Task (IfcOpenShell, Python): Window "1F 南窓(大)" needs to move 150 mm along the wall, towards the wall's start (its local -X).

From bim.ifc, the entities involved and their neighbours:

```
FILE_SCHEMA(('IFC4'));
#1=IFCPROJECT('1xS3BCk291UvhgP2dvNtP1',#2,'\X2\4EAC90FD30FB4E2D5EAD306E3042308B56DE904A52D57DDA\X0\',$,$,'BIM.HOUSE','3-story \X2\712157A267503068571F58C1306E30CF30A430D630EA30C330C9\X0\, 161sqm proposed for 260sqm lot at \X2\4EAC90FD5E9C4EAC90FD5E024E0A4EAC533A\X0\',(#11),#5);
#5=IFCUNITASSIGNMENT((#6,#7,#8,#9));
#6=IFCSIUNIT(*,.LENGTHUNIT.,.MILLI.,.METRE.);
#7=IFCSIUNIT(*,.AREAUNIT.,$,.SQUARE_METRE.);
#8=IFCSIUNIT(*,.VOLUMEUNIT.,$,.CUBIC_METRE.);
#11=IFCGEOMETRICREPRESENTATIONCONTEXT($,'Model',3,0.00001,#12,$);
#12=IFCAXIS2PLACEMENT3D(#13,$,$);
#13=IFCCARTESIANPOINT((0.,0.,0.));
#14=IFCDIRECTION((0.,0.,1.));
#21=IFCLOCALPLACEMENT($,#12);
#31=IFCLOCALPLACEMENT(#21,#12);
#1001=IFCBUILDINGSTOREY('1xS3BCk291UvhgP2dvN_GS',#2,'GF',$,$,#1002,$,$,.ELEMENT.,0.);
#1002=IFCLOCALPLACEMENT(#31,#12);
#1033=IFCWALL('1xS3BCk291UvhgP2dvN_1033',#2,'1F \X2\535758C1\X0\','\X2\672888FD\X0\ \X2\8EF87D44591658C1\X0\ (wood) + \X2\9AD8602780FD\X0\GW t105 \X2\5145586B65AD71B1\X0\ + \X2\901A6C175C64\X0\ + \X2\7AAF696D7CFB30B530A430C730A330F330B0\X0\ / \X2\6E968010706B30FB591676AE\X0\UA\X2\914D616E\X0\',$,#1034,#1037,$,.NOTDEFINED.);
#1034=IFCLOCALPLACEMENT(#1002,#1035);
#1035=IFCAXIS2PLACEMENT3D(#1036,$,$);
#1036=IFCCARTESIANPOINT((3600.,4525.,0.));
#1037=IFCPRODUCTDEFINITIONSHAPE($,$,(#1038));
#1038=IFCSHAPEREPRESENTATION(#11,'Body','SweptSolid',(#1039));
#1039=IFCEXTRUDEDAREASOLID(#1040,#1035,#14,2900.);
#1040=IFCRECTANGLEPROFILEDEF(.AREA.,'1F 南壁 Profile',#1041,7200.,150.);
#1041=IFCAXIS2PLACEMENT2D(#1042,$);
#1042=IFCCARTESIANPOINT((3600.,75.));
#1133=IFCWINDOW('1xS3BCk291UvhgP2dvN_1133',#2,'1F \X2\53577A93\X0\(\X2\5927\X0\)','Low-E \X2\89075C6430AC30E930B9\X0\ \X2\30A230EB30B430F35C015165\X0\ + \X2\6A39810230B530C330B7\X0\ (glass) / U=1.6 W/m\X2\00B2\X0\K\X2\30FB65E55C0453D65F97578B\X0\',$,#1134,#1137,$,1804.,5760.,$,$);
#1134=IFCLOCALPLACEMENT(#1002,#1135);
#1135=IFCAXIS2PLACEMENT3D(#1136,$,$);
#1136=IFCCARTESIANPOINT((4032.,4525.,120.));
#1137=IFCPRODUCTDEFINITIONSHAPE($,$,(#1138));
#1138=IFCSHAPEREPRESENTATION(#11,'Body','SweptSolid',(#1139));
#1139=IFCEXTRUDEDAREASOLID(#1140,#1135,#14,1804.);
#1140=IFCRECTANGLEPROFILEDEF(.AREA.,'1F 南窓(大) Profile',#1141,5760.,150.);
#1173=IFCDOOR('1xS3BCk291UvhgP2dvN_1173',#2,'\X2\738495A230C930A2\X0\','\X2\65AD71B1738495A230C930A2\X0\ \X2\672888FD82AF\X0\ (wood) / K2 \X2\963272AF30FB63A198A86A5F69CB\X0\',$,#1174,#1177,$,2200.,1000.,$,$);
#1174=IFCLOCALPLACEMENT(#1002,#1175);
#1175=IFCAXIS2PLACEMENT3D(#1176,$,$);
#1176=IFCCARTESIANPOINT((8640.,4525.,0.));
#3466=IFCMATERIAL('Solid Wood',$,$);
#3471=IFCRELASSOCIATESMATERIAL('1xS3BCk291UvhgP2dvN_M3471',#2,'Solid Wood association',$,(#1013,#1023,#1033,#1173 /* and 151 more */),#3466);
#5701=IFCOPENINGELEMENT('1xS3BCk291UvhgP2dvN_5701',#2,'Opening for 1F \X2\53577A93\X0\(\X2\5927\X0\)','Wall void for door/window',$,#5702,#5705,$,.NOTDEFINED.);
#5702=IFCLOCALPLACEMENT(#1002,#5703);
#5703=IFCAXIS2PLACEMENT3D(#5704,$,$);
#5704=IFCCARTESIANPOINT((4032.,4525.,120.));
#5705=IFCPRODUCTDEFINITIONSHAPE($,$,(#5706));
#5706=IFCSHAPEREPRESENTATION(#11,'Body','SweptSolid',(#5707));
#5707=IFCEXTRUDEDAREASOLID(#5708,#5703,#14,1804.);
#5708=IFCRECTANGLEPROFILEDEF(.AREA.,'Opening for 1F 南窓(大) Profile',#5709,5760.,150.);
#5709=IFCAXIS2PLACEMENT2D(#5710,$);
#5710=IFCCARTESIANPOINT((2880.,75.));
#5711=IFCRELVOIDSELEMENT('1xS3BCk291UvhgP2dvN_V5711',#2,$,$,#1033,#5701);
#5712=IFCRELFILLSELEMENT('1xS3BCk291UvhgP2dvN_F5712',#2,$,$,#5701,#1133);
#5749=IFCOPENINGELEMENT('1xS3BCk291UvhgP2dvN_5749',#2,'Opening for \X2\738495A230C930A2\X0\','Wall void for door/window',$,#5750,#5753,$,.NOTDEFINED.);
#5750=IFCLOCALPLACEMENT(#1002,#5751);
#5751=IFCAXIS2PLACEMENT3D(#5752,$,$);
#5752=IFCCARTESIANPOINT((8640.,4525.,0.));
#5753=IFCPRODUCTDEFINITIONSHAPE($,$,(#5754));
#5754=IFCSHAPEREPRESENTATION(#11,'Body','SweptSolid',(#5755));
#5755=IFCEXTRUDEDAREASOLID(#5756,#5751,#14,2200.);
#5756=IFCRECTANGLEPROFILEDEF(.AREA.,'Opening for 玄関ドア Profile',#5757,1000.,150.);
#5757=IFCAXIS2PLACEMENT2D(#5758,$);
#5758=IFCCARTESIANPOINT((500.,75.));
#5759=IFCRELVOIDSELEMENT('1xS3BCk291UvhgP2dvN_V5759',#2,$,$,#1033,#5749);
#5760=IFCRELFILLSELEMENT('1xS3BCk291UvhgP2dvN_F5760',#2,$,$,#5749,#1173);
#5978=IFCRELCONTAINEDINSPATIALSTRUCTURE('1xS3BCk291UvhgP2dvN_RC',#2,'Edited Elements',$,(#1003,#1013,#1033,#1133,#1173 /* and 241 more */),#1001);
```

```python
import ifcopenshell
import ifcopenshell.api.geometry
import ifcopenshell.util.placement

model = ifcopenshell.open("bim.ifc")

window = model.by_guid("1xS3BCk291UvhgP2dvN_1133")
opening = window.FillsVoids[0].RelatingOpeningElement
wall = opening.VoidsElements[0].RelatingBuildingElement

wall_matrix = ifcopenshell.util.placement.get_local_placement(wall.ObjectPlacement)
shift = wall_matrix[:3, 0] * -150.0
before = ifcopenshell.util.placement.get_local_placement(window.ObjectPlacement)[:3, 3].copy()

# The window is not placed relative to its opening, so move both.
for product in (opening, window):
    matrix = ifcopenshell.util.placement.get_local_placement(product.ObjectPlacement)
    matrix[:3, 3] += shift
    ifcopenshell.api.geometry.edit_object_placement(model, product=product, matrix=matrix, is_si=False)

after = ifcopenshell.util.placement.get_local_placement(window.ObjectPlacement)[:3, 3]
print("window moved by", (after - before).round(3) + 0.0)

model.write("bim_rev.ifc")
```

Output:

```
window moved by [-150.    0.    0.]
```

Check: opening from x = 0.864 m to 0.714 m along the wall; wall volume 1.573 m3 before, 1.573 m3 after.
